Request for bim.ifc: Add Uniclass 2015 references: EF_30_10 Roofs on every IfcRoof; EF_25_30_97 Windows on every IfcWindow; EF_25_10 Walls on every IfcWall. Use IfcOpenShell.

First a look at what the model holds.

```python
import ifcopenshell

model = ifcopenshell.open("bim.ifc")
print(model.schema)
print("classifications:", [c.Name for c in model.by_type("IfcClassification")])
for ifc_class in ("IfcDoor", "IfcRoof", "IfcStair", "IfcWall", "IfcWindow"):
    print(ifc_class, len(model.by_type(ifc_class)))
```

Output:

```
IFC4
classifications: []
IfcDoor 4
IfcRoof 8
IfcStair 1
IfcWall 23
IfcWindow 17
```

```python
import ifcopenshell
import ifcopenshell.api.classification

model = ifcopenshell.open("bim.ifc")

system = ifcopenshell.api.classification.add_classification(model, classification="Uniclass 2015")

codes = {
    "IfcRoof": ("EF_30_10", "Roofs"),
    "IfcWindow": ("EF_25_30_97", "Windows"),
    "IfcWall": ("EF_25_10", "Walls"),
}
for ifc_class, (code, name) in codes.items():
    products = model.by_type(ifc_class)
    ifcopenshell.api.classification.add_reference(
        model, products=products, classification=system, identification=code, name=name
    )
    print(code, len(products))

model.write("bim_updated.ifc")
```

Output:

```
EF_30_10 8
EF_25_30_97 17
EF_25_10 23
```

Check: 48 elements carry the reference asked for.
